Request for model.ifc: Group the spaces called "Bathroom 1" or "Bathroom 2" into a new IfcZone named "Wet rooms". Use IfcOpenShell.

First a look at what the model holds.

```python
import ifcopenshell

model = ifcopenshell.open("model.ifc")
print(model.schema)
seen = {}
for space in model.by_type("IfcSpace"):
    seen[space.LongName] = seen.get(space.LongName, 0) + 1
for name, count in sorted(seen.items(), key=str):
    print(count, "x", name)
print("zones:", [z.Name for z in model.by_type("IfcZone")][:20])
```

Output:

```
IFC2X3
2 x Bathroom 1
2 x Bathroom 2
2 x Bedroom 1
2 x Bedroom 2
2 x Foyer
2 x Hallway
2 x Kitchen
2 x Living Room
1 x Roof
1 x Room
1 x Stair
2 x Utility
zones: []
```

```python
import ifcopenshell
import ifcopenshell.api.group
import ifcopenshell.api.root

model = ifcopenshell.open("model.ifc")

names = {"Bathroom 1", "Bathroom 2"}
spaces = [s for s in model.by_type("IfcSpace") if s.LongName in names]

zone = ifcopenshell.api.root.create_entity(model, ifc_class="IfcZone", name="Wet rooms")
ifcopenshell.api.group.assign_group(model, products=spaces, group=zone)
print(len(spaces), "spaces in", zone.Name)

model.write("model_v2.ifc")
```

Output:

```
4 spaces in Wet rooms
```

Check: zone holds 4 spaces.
